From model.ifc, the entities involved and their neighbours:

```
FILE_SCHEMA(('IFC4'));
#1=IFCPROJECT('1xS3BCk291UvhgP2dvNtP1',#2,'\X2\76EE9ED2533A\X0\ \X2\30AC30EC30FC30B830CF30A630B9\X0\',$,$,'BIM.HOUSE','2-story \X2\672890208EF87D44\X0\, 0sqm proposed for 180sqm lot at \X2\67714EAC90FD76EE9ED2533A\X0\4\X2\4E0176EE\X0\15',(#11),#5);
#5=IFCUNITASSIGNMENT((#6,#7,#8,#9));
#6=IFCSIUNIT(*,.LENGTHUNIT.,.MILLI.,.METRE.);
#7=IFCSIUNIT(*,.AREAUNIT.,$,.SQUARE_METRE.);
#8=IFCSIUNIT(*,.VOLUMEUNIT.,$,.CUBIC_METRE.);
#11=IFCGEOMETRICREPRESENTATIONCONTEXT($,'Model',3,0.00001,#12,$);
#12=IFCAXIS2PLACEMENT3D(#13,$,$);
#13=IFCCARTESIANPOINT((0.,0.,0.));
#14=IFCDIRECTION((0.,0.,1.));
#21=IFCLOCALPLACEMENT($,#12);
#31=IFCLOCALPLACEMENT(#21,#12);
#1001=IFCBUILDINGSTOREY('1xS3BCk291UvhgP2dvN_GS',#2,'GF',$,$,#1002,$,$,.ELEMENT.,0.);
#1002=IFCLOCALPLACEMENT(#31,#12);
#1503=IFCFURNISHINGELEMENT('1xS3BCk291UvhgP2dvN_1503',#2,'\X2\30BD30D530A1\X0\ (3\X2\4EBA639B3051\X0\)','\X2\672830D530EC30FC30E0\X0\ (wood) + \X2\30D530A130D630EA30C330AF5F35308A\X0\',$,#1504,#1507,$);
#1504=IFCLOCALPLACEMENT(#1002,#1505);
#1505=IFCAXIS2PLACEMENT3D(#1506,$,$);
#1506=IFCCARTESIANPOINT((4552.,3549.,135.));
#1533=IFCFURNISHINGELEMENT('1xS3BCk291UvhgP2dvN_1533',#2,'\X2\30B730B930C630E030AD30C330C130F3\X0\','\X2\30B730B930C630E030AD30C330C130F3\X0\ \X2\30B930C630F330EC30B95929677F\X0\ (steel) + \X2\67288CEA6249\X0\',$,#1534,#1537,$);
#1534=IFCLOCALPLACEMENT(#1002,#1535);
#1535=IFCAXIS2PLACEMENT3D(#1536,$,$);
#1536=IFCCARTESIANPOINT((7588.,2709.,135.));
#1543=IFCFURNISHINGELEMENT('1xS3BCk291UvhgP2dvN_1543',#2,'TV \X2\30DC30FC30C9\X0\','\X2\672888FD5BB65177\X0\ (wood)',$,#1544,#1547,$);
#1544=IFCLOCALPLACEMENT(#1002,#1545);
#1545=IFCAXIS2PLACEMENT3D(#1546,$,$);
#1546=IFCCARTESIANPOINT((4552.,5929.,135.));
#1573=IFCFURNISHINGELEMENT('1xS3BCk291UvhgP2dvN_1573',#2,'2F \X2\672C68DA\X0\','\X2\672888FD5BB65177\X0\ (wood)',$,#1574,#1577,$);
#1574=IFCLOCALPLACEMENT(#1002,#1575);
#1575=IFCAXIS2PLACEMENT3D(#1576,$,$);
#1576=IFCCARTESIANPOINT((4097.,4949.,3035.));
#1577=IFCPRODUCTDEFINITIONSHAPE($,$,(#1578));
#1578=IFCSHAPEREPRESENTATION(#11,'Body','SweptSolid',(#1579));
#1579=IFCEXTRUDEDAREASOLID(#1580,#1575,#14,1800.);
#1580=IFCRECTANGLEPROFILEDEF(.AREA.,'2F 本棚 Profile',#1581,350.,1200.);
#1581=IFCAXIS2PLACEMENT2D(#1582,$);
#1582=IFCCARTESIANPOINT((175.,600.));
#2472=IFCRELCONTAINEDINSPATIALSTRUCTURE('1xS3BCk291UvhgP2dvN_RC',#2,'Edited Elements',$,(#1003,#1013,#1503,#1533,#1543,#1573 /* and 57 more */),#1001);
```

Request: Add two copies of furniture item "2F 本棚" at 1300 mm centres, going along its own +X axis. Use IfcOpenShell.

```python
import ifcopenshell
import ifcopenshell.api.geometry
import ifcopenshell.api.root
import ifcopenshell.util.element
import ifcopenshell.util.placement

model = ifcopenshell.open("model.ifc")


def reuse_history(source, copy):
    """copy_class also copies each property set's owner history, people and application; keep the originals."""
    for rel in copy.IsDefinedBy:
        if rel.is_a("IfcRelDefinesByProperties") and (history := rel.RelatingPropertyDefinition.OwnerHistory):
            rel.RelatingPropertyDefinition.OwnerHistory = source.OwnerHistory
            ifcopenshell.util.element.remove_deep2(model, history)


source = model.by_guid("1xS3BCk291UvhgP2dvN_1573")
base = ifcopenshell.util.placement.get_local_placement(source.ObjectPlacement)
step = base[:3, 0] * 1300.0

for i in range(1, 3):
    copy = ifcopenshell.api.root.copy_class(model, product=source)
    copy.Representation = ifcopenshell.util.element.copy_deep(
        model, source.Representation, exclude=["IfcGeometricRepresentationContext", "IfcRepresentationMap"]
    )
    reuse_history(source, copy)
    matrix = base.copy()
    matrix[:3, 3] += i * step
    print("added at", matrix[:3, 3].round(3) + 0.0)
    ifcopenshell.api.geometry.edit_object_placement(model, product=copy, matrix=matrix, is_si=False)

model.write("model_updated.ifc")
```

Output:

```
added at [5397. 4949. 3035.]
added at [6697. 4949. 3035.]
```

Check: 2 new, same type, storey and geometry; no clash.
